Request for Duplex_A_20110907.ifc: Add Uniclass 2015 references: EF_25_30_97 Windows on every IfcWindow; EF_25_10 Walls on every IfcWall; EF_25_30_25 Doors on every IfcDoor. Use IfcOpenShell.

First a look at what the model holds.

```python
import ifcopenshell

model = ifcopenshell.open("Duplex_A_20110907.ifc")
print(model.schema)
print("classifications:", [c.Name for c in model.by_type("IfcClassification")])
for ifc_class in ("IfcDoor", "IfcRoof", "IfcStair", "IfcWall", "IfcWindow"):
    print(ifc_class, len(model.by_type(ifc_class)))
```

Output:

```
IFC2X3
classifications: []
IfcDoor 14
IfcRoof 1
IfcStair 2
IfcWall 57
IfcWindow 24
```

```python
import ifcopenshell
import ifcopenshell.api.classification

model = ifcopenshell.open("Duplex_A_20110907.ifc")

# IFC2X3 requires Source and Edition and has no link from the project to the system.
system = model.create_entity("IfcClassification", Source="NBS", Edition="2015", Name="Uniclass 2015")

codes = {
    "IfcWindow": ("EF_25_30_97", "Windows"),
    "IfcWall": ("EF_25_10", "Walls"),
    "IfcDoor": ("EF_25_30_25", "Doors"),
}
for ifc_class, (code, name) in codes.items():
    products = model.by_type(ifc_class)
    ifcopenshell.api.classification.add_reference(
        model, products=products, classification=system, identification=code, name=name
    )
    print(code, len(products))

model.write("Duplex_A_20110907_v2.ifc")
```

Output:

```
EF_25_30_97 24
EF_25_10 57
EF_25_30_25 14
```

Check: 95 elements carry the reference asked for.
